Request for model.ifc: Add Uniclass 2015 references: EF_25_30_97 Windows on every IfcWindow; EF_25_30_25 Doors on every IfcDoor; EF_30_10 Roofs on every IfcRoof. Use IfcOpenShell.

First a look at what the model holds.

```python
import ifcopenshell

model = ifcopenshell.open("model.ifc")
print(model.schema)
print("classifications:", [c.Name for c in model.by_type("IfcClassification")])
for ifc_class in ("IfcDoor", "IfcRoof", "IfcStair", "IfcWall", "IfcWindow"):
    print(ifc_class, len(model.by_type(ifc_class)))
```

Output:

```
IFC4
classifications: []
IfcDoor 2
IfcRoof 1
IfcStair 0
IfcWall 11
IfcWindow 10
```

```python
import ifcopenshell
import ifcopenshell.api.classification

model = ifcopenshell.open("model.ifc")

system = ifcopenshell.api.classification.add_classification(model, classification="Uniclass 2015")

codes = {
    "IfcWindow": ("EF_25_30_97", "Windows"),
    "IfcDoor": ("EF_25_30_25", "Doors"),
    "IfcRoof": ("EF_30_10", "Roofs"),
}
for ifc_class, (code, name) in codes.items():
    products = model.by_type(ifc_class)
    ifcopenshell.api.classification.add_reference(
        model, products=products, classification=system, identification=code, name=name
    )
    print(code, len(products))

model.write("model_v2.ifc")
```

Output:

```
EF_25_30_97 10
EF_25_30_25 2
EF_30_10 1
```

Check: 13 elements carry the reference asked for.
